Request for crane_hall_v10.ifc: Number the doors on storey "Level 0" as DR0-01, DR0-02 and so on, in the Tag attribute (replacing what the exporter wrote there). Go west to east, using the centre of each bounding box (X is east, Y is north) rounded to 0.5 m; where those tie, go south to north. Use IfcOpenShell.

First a look at what the model holds.

```python
import ifcopenshell
import ifcopenshell.util.element
import ifcopenshell.util.placement

model = ifcopenshell.open("crane_hall_v10.ifc")
print(model.schema)
storey = next(s for s in model.by_type("IfcBuildingStorey") if s.Name == "Level 0")
doors = [e for e in ifcopenshell.util.element.get_decomposition(storey) if e.is_a("IfcDoor")]
for e in sorted(doors, key=lambda e: e.id()):
    origin = ifcopenshell.util.placement.get_local_placement(e.ObjectPlacement)[:3, 3]
    print(e.id(), e.Tag, e.Name, origin.round(2) + 0.0, sep=" | ")
```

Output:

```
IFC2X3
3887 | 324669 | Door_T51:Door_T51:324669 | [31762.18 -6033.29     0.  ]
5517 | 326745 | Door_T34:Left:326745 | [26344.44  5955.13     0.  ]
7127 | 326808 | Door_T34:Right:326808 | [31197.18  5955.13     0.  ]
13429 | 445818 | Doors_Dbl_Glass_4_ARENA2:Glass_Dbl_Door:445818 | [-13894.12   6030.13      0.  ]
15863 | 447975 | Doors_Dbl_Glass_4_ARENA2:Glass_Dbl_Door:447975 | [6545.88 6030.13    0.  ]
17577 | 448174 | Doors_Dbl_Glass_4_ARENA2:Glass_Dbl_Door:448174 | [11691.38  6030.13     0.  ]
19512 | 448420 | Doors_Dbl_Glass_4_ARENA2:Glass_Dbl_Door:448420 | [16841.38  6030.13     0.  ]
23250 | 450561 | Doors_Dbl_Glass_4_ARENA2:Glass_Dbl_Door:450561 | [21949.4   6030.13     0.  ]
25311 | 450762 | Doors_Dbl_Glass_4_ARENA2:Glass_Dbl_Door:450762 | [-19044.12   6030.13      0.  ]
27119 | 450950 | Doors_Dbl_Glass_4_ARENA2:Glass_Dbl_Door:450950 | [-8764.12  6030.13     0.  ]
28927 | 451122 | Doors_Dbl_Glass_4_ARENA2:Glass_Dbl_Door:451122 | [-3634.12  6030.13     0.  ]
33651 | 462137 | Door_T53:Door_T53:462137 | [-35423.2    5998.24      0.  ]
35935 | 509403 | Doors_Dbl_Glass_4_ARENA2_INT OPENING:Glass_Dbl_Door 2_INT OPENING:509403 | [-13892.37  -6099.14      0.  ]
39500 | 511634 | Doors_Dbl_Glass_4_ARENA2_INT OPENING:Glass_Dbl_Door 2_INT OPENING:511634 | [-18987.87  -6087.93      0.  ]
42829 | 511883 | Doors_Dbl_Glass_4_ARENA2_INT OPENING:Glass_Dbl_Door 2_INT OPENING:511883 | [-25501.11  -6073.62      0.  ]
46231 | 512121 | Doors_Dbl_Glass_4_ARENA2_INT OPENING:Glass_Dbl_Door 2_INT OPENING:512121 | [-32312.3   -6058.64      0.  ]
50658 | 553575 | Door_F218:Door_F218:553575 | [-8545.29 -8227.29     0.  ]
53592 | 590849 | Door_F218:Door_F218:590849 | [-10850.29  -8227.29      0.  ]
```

```python
import ifcopenshell
import ifcopenshell.geom
import ifcopenshell.util.element
import ifcopenshell.util.shape

model = ifcopenshell.open("crane_hall_v10.ifc")
settings = ifcopenshell.geom.settings()
settings.set("use-world-coords", True)


def centre(element):
    shape = ifcopenshell.geom.create_shape(settings, element)
    return ifcopenshell.util.shape.get_bbox_centroid(shape.geometry)


storey = next(s for s in model.by_type("IfcBuildingStorey") if s.Name == "Level 0")
doors = [e for e in ifcopenshell.util.element.get_decomposition(storey) if e.is_a("IfcDoor")]

# Insertion points can sit at a corner or the storey origin, so sort by the geometry (in metres).
centres = {e: centre(e) for e in doors}
doors.sort(key=lambda e: (round(centres[e][0] / 0.5), centres[e][1]))

for i, e in enumerate(doors, start=1):
    number = f"DR0-{i:02d}"
    e.Tag = number
    print(e.id(), number)

model.write("crane_hall_v10-out.ifc")
```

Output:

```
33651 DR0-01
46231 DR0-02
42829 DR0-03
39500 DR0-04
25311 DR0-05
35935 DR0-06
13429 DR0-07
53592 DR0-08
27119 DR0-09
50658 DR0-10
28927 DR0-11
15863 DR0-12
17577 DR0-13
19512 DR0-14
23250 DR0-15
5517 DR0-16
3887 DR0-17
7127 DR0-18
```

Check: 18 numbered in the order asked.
